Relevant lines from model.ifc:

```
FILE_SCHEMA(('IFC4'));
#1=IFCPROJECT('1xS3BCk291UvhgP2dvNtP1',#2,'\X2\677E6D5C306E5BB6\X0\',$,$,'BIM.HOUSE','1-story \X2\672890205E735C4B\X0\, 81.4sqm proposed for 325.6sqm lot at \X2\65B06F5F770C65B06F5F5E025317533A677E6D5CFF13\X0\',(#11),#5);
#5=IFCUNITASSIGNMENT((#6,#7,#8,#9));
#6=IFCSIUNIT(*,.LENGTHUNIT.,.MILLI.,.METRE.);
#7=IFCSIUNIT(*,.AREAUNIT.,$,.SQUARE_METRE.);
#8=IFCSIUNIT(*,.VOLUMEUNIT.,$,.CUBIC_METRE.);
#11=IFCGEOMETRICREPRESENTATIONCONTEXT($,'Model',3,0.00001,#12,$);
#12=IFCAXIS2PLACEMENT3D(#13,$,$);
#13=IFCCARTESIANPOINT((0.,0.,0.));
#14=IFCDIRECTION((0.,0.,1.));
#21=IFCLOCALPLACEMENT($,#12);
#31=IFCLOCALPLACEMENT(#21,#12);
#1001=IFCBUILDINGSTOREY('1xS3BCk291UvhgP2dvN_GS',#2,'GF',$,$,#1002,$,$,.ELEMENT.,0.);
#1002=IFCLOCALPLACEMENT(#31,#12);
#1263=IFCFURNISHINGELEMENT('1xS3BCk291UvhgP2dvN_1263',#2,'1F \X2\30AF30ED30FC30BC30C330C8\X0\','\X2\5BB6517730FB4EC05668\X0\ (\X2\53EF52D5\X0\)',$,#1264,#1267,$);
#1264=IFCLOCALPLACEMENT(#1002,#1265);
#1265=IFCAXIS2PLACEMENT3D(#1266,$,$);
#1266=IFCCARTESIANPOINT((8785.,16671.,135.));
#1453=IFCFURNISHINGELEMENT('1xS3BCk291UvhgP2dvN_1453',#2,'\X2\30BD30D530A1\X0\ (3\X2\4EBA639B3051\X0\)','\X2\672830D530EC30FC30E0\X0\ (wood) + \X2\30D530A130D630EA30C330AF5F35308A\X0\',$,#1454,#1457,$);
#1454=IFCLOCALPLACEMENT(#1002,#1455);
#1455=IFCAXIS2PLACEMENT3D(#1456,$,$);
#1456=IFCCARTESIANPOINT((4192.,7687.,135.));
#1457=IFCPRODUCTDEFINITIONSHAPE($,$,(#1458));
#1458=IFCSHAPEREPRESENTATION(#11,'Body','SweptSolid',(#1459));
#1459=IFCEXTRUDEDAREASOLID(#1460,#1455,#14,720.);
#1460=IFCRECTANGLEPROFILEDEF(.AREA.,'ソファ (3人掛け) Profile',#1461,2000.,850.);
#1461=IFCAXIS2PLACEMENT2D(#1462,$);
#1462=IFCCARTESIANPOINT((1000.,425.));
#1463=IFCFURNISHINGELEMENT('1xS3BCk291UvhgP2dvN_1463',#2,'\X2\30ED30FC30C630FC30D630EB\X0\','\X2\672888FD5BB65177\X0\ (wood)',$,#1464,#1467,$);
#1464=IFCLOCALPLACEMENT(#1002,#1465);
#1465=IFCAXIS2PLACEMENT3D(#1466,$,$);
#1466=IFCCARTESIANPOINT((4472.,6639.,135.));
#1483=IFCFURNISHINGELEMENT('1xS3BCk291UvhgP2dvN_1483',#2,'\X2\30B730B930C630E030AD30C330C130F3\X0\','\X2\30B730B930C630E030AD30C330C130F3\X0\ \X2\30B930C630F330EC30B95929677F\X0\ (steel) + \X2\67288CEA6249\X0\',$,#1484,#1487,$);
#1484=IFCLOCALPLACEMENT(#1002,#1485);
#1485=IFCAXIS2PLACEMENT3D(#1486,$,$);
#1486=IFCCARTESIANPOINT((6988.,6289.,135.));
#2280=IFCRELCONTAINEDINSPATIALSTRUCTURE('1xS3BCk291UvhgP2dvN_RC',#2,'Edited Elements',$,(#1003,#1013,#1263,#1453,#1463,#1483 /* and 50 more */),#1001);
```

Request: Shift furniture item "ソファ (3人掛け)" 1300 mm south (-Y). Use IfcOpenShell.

```python
import ifcopenshell
import ifcopenshell.api.geometry
import ifcopenshell.util.placement

model = ifcopenshell.open("model.ifc")

item = model.by_guid("1xS3BCk291UvhgP2dvN_1453")
matrix = ifcopenshell.util.placement.get_local_placement(item.ObjectPlacement)
matrix[1, 3] -= 1300.0
ifcopenshell.api.geometry.edit_object_placement(model, product=item, matrix=matrix, is_si=False)

print(ifcopenshell.util.placement.get_local_placement(item.ObjectPlacement).round(3) + 0.0)

model.write("model_rev.ifc")
```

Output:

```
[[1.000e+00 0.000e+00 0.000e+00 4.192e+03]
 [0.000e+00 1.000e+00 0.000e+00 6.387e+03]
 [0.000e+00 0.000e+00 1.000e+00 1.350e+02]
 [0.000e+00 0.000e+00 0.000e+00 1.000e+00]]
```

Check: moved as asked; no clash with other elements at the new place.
